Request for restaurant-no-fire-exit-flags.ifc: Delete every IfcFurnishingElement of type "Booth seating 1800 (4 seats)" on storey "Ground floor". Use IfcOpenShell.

First a look at what the model holds.

```python
import ifcopenshell
import ifcopenshell.util.element

model = ifcopenshell.open("restaurant-no-fire-exit-flags.ifc")
print(model.schema)
storey = next(s for s in model.by_type("IfcBuildingStorey") if s.Name == "Ground floor")
furniture = [e for e in ifcopenshell.util.element.get_decomposition(storey) if e.is_a("IfcFurnishingElement")]
seen = {}
for e in furniture:
    element_type = ifcopenshell.util.element.get_type(e)
    name = element_type.Name if element_type not in (None, e) else None
    seen[name] = seen.get(name, 0) + 1
for name, count in sorted(seen.items(), key=str):
    print(count, "x", name)
```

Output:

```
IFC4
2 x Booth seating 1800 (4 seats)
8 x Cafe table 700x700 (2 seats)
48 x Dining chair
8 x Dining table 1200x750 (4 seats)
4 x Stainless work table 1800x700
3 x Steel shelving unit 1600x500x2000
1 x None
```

```python
import ifcopenshell
import ifcopenshell.api.root
import ifcopenshell.util.element

model = ifcopenshell.open("restaurant-no-fire-exit-flags.ifc")

storey = next(s for s in model.by_type("IfcBuildingStorey") if s.Name == "Ground floor")
furniture = [e for e in ifcopenshell.util.element.get_decomposition(storey) if e.is_a("IfcFurnishingElement")]
targets = [e for e in furniture if (t := ifcopenshell.util.element.get_type(e)) not in (None, e) and t.Name == "Booth seating 1800 (4 seats)"]

for e in targets:
    ifcopenshell.api.root.remove_product(model, product=e)
print(len(targets), "removed")

model.write("restaurant-no-fire-exit-flags_rev.ifc")
```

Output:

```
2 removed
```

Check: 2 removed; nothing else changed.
